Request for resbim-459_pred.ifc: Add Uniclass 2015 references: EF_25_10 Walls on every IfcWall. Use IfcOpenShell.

First a look at what the model holds.

```python
import ifcopenshell

model = ifcopenshell.open("resbim-459_pred.ifc")
print(model.schema)
print("classifications:", [c.Name for c in model.by_type("IfcClassification")])
for ifc_class in ("IfcDoor", "IfcRoof", "IfcStair", "IfcWall", "IfcWindow"):
    print(ifc_class, len(model.by_type(ifc_class)))
```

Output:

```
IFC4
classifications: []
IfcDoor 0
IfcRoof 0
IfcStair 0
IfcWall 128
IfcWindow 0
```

```python
import ifcopenshell
import ifcopenshell.api.classification

model = ifcopenshell.open("resbim-459_pred.ifc")

system = ifcopenshell.api.classification.add_classification(model, classification="Uniclass 2015")

codes = {
    "IfcWall": ("EF_25_10", "Walls"),
}
for ifc_class, (code, name) in codes.items():
    products = model.by_type(ifc_class)
    ifcopenshell.api.classification.add_reference(
        model, products=products, classification=system, identification=code, name=name
    )
    print(code, len(products))

model.write("resbim-459_pred_updated.ifc")
```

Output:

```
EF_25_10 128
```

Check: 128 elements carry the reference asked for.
